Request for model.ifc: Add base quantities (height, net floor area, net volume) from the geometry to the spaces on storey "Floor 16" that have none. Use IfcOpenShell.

First a look at what the model holds.

```python
import ifcopenshell
import ifcopenshell.util.element
import ifcopenshell.util.unit

model = ifcopenshell.open("model.ifc")
print(model.schema)
for unit_type in ("LENGTHUNIT", "AREAUNIT", "VOLUMEUNIT"):
    print(unit_type, ifcopenshell.util.unit.calculate_unit_scale(model, unit_type))
storey = next(s for s in model.by_type("IfcBuildingStorey") if s.Name == "Floor 16")
spaces = [e for e in ifcopenshell.util.element.get_decomposition(storey) if e.is_a("IfcSpace")]
for e in sorted(spaces, key=lambda e: e.id()):
    print(e.id(), e.is_a(), e.Name, list(ifcopenshell.util.element.get_psets(e, qtos_only=True)), sep=" | ")
```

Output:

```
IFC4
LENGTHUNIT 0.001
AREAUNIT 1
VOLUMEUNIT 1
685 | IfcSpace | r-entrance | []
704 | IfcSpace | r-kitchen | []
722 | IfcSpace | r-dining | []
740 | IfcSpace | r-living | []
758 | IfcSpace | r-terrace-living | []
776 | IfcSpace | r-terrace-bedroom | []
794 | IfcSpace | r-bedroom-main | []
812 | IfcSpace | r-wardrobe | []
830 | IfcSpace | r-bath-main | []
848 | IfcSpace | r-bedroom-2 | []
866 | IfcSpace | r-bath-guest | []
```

```python
import ifcopenshell
import ifcopenshell.api.pset
import ifcopenshell.geom
import ifcopenshell.util.element
import ifcopenshell.util.shape
import ifcopenshell.util.unit

model = ifcopenshell.open("model.ifc")
unit_scale = ifcopenshell.util.unit.calculate_unit_scale(model)
area_scale = ifcopenshell.util.unit.calculate_unit_scale(model, "AREAUNIT")
volume_scale = ifcopenshell.util.unit.calculate_unit_scale(model, "VOLUMEUNIT")
settings = ifcopenshell.geom.settings()

storey = next(s for s in model.by_type("IfcBuildingStorey") if s.Name == "Floor 16")
spaces = [e for e in ifcopenshell.util.element.get_decomposition(storey) if e.is_a("IfcSpace")]

for e in sorted(spaces, key=lambda e: e.id()):
    if ifcopenshell.util.element.get_psets(e, qtos_only=True, should_inherit=False):
        continue
    # Geometry comes back in metres, in the element's own axes.
    shape = ifcopenshell.geom.create_shape(settings, e)
    values = {
        "Height": ifcopenshell.util.shape.get_z(shape.geometry) / unit_scale,
        "NetFloorArea": ifcopenshell.util.shape.get_footprint_area(shape.geometry) / area_scale,
        "NetVolume": ifcopenshell.util.shape.get_volume(shape.geometry) / volume_scale,
    }
    qto = ifcopenshell.api.pset.add_qto(model, product=e, name="Qto_SpaceBaseQuantities")
    ifcopenshell.api.pset.edit_qto(model, qto=qto, properties=values)
    print(e.id(), {k: round(v, 3) for k, v in values.items()})

model.write("model-out.ifc")
```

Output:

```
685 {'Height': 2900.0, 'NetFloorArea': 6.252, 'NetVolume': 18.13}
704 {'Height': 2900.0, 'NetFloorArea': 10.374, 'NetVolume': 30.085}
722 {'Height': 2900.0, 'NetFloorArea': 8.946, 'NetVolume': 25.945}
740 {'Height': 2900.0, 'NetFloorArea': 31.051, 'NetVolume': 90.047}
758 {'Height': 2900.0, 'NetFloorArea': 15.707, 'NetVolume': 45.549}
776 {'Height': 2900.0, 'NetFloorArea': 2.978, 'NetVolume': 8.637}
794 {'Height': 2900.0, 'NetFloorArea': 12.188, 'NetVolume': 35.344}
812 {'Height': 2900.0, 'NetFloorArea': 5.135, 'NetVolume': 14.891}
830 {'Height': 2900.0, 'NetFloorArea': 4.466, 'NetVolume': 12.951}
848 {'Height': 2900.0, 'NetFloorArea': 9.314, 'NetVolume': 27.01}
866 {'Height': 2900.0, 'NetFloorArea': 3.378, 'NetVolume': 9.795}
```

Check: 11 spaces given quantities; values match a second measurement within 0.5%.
